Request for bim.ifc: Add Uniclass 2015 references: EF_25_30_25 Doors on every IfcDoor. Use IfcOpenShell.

First a look at what the model holds.

```python
import ifcopenshell

model = ifcopenshell.open("bim.ifc")
print(model.schema)
print("classifications:", [c.Name for c in model.by_type("IfcClassification")])
for ifc_class in ("IfcDoor", "IfcRoof", "IfcStair", "IfcWall", "IfcWindow"):
    print(ifc_class, len(model.by_type(ifc_class)))
```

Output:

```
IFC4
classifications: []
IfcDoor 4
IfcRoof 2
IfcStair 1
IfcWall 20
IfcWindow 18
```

```python
import ifcopenshell
import ifcopenshell.api.classification

model = ifcopenshell.open("bim.ifc")

system = ifcopenshell.api.classification.add_classification(model, classification="Uniclass 2015")

codes = {
    "IfcDoor": ("EF_25_30_25", "Doors"),
}
for ifc_class, (code, name) in codes.items():
    products = model.by_type(ifc_class)
    ifcopenshell.api.classification.add_reference(
        model, products=products, classification=system, identification=code, name=name
    )
    print(code, len(products))

model.write("bim-out.ifc")
```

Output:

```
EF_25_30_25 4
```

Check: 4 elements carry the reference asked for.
